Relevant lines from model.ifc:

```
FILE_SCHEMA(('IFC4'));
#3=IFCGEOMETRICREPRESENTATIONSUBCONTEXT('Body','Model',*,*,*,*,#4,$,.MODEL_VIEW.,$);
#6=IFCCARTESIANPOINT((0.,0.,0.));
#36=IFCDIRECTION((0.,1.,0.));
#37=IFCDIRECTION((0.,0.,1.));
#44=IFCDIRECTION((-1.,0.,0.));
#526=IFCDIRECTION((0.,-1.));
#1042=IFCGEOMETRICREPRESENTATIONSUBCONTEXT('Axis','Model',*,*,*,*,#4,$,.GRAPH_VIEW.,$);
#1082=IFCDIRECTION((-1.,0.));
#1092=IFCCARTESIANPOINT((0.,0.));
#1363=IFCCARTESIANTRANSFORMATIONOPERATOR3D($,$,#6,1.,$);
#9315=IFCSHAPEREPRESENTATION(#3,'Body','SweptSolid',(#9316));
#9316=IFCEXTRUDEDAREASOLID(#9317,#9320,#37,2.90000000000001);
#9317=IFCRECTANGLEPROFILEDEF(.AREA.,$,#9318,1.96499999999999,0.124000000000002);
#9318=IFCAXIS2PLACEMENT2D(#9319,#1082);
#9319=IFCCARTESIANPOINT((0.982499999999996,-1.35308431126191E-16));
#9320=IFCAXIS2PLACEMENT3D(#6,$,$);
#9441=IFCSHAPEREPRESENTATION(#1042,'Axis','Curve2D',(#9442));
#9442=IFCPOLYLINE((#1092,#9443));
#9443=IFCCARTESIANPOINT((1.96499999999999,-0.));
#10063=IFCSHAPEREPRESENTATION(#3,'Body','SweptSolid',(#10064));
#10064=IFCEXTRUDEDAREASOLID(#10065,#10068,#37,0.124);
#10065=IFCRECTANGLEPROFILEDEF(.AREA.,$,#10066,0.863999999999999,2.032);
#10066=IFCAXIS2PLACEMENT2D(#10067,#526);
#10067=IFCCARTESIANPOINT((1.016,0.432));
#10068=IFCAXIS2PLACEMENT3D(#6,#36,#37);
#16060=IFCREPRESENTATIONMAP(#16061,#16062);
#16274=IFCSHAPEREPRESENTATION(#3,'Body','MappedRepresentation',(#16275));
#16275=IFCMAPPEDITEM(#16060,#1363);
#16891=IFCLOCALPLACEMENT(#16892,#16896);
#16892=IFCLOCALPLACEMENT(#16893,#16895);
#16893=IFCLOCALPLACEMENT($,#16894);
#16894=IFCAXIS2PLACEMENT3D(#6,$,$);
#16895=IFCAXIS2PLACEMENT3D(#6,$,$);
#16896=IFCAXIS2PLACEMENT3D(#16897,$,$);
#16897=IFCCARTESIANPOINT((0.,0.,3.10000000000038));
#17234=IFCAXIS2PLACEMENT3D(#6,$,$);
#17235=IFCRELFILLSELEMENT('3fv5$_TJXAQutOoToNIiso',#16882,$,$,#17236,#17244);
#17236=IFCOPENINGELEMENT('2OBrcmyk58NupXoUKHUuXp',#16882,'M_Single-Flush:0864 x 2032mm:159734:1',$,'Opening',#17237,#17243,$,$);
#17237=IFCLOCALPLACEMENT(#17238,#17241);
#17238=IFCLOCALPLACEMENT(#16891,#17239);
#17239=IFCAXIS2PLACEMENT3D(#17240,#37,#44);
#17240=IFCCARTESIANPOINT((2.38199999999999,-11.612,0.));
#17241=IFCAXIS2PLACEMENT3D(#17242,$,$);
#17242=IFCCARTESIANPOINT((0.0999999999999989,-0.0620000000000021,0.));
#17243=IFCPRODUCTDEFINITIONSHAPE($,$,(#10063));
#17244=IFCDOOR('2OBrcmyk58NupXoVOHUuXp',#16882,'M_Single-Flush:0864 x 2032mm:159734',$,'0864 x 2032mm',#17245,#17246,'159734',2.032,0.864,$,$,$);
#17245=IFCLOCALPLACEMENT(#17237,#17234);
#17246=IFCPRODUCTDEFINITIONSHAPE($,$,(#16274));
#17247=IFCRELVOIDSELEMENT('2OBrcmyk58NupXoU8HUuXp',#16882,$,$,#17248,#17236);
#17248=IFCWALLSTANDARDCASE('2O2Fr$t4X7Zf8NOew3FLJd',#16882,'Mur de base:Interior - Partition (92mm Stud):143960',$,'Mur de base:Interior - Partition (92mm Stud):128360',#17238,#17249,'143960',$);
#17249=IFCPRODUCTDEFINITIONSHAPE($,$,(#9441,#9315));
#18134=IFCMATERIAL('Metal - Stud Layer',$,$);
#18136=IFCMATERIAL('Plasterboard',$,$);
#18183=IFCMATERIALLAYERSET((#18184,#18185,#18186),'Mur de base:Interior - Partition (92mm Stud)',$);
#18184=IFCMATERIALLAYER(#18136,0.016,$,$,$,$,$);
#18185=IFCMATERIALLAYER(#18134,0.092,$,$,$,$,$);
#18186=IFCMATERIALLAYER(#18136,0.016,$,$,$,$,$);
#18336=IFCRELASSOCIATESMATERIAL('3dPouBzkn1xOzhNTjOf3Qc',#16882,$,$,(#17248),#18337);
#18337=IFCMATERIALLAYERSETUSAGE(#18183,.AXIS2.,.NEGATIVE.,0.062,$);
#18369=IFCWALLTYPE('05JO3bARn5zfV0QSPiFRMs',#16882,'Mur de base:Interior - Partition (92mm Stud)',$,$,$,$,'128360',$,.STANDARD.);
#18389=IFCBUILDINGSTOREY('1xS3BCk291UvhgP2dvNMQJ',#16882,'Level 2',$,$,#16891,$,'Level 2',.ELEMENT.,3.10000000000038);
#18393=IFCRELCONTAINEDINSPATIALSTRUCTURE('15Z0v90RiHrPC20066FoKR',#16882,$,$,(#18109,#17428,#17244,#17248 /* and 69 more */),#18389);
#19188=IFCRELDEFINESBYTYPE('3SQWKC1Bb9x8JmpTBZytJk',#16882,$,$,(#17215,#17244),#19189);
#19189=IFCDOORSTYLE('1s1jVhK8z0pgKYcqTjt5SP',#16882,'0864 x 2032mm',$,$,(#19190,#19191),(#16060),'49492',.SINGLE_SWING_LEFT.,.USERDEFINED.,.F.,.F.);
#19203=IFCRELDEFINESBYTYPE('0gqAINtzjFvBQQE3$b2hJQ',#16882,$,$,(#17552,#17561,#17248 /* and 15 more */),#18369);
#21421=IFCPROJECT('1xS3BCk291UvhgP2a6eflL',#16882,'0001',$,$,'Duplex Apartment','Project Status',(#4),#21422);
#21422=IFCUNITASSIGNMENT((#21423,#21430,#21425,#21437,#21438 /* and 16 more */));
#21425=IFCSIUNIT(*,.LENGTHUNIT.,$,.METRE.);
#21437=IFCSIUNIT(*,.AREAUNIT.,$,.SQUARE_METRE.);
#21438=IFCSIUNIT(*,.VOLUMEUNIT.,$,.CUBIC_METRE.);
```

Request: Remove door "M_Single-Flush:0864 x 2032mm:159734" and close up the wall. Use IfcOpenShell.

```python
import ifcopenshell
import ifcopenshell.api.feature
import ifcopenshell.api.root
import ifcopenshell.geom
import ifcopenshell.util.shape

model = ifcopenshell.open("model.ifc")
settings = ifcopenshell.geom.settings()


def volume(element):
    """Net volume in cubic metres, openings subtracted."""
    shape = ifcopenshell.geom.create_shape(settings, element)
    return ifcopenshell.util.shape.get_volume(shape.geometry)


door = model.by_guid("2OBrcmyk58NupXoVOHUuXp")
opening = door.FillsVoids[0].RelatingOpeningElement
wall = opening.VoidsElements[0].RelatingBuildingElement
before = volume(wall)

ifcopenshell.api.root.remove_product(model, product=door)
ifcopenshell.api.feature.remove_feature(model, feature=opening)

after = volume(wall)

print(f"wall volume {before:.3f} -> {after:.3f} m3")

model.write("model-out.ifc")
```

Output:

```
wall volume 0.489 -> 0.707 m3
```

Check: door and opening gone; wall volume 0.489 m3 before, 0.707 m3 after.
